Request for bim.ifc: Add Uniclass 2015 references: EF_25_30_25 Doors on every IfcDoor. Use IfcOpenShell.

First a look at what the model holds.

```python
import ifcopenshell

model = ifcopenshell.open("bim.ifc")
print(model.schema)
print("classifications:", [c.Name for c in model.by_type("IfcClassification")])
for ifc_class in ("IfcDoor", "IfcRoof", "IfcStair", "IfcWall", "IfcWindow"):
    print(ifc_class, len(model.by_type(ifc_class)))
```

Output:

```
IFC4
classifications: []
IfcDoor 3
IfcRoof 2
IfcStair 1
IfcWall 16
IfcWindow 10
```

```python
import ifcopenshell
import ifcopenshell.api.classification

model = ifcopenshell.open("bim.ifc")

system = ifcopenshell.api.classification.add_classification(model, classification="Uniclass 2015")

codes = {
    "IfcDoor": ("EF_25_30_25", "Doors"),
}
for ifc_class, (code, name) in codes.items():
    products = model.by_type(ifc_class)
    ifcopenshell.api.classification.add_reference(
        model, products=products, classification=system, identification=code, name=name
    )
    print(code, len(products))

model.write("bim_edited.ifc")
```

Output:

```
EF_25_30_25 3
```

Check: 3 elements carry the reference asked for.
